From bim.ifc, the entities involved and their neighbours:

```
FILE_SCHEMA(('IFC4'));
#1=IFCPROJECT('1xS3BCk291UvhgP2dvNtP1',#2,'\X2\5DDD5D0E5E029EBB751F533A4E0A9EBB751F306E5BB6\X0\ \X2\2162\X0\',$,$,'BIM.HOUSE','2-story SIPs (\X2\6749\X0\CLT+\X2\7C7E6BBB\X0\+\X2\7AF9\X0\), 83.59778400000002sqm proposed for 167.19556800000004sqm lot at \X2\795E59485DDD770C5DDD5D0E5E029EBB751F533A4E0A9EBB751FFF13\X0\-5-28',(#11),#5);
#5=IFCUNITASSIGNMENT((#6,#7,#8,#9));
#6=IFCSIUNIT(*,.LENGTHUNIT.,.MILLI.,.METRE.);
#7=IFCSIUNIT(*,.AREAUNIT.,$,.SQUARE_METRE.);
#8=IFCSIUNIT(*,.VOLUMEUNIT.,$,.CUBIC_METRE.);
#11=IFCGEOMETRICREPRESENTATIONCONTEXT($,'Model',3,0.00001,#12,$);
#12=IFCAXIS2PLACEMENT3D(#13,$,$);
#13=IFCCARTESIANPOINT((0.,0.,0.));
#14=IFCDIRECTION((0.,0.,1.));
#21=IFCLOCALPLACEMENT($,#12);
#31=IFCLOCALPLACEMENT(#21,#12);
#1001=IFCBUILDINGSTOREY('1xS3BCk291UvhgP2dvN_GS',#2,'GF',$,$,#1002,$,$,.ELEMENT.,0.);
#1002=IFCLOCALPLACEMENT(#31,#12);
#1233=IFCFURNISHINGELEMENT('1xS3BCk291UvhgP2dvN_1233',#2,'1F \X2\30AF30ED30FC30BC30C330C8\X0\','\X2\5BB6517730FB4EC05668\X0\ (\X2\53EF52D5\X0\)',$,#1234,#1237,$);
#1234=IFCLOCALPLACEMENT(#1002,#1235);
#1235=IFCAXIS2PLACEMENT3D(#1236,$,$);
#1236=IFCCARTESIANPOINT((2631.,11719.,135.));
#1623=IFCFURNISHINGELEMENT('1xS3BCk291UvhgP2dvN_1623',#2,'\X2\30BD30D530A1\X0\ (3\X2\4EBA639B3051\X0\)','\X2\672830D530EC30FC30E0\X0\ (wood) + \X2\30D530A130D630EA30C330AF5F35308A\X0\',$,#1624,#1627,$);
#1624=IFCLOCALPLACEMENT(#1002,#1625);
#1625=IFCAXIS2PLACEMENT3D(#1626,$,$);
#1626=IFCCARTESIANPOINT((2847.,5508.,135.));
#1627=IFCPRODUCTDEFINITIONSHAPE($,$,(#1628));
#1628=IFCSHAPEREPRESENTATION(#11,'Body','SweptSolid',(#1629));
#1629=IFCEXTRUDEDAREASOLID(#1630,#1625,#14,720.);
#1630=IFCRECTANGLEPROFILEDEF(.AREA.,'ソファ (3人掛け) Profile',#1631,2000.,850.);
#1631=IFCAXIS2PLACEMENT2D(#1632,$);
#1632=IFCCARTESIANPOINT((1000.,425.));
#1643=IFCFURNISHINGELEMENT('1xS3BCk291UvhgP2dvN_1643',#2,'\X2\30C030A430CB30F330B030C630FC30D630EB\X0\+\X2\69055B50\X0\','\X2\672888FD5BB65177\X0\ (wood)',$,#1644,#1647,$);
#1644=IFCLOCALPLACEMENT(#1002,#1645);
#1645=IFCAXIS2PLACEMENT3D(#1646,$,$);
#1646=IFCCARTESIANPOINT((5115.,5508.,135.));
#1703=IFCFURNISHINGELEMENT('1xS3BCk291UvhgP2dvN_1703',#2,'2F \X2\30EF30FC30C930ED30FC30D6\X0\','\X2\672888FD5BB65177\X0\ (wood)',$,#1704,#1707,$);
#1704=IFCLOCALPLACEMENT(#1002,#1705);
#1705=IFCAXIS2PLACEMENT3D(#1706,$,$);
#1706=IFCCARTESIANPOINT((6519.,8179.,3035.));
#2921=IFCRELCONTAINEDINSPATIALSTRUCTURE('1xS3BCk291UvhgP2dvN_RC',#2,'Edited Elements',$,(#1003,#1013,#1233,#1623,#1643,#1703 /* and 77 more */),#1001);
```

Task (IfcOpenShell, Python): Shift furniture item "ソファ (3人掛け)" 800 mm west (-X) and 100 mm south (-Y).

```python
import ifcopenshell
import ifcopenshell.api.geometry
import ifcopenshell.util.placement
import ifcopenshell.util.unit

model = ifcopenshell.open("bim.ifc")
unit_scale = ifcopenshell.util.unit.calculate_unit_scale(model)

item = model.by_guid("1xS3BCk291UvhgP2dvN_1623")
matrix = ifcopenshell.util.placement.get_local_placement(item.ObjectPlacement)
matrix[0, 3] -= 0.8 / unit_scale
matrix[1, 3] -= 0.1 / unit_scale
ifcopenshell.api.geometry.edit_object_placement(model, product=item, matrix=matrix, is_si=False)

print(ifcopenshell.util.placement.get_local_placement(item.ObjectPlacement).round(3) + 0.0)

model.write("bim-out.ifc")
```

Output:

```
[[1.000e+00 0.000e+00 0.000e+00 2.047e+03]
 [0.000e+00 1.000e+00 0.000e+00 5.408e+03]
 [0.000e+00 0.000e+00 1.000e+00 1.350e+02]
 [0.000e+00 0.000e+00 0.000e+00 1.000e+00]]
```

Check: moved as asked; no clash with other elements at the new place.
